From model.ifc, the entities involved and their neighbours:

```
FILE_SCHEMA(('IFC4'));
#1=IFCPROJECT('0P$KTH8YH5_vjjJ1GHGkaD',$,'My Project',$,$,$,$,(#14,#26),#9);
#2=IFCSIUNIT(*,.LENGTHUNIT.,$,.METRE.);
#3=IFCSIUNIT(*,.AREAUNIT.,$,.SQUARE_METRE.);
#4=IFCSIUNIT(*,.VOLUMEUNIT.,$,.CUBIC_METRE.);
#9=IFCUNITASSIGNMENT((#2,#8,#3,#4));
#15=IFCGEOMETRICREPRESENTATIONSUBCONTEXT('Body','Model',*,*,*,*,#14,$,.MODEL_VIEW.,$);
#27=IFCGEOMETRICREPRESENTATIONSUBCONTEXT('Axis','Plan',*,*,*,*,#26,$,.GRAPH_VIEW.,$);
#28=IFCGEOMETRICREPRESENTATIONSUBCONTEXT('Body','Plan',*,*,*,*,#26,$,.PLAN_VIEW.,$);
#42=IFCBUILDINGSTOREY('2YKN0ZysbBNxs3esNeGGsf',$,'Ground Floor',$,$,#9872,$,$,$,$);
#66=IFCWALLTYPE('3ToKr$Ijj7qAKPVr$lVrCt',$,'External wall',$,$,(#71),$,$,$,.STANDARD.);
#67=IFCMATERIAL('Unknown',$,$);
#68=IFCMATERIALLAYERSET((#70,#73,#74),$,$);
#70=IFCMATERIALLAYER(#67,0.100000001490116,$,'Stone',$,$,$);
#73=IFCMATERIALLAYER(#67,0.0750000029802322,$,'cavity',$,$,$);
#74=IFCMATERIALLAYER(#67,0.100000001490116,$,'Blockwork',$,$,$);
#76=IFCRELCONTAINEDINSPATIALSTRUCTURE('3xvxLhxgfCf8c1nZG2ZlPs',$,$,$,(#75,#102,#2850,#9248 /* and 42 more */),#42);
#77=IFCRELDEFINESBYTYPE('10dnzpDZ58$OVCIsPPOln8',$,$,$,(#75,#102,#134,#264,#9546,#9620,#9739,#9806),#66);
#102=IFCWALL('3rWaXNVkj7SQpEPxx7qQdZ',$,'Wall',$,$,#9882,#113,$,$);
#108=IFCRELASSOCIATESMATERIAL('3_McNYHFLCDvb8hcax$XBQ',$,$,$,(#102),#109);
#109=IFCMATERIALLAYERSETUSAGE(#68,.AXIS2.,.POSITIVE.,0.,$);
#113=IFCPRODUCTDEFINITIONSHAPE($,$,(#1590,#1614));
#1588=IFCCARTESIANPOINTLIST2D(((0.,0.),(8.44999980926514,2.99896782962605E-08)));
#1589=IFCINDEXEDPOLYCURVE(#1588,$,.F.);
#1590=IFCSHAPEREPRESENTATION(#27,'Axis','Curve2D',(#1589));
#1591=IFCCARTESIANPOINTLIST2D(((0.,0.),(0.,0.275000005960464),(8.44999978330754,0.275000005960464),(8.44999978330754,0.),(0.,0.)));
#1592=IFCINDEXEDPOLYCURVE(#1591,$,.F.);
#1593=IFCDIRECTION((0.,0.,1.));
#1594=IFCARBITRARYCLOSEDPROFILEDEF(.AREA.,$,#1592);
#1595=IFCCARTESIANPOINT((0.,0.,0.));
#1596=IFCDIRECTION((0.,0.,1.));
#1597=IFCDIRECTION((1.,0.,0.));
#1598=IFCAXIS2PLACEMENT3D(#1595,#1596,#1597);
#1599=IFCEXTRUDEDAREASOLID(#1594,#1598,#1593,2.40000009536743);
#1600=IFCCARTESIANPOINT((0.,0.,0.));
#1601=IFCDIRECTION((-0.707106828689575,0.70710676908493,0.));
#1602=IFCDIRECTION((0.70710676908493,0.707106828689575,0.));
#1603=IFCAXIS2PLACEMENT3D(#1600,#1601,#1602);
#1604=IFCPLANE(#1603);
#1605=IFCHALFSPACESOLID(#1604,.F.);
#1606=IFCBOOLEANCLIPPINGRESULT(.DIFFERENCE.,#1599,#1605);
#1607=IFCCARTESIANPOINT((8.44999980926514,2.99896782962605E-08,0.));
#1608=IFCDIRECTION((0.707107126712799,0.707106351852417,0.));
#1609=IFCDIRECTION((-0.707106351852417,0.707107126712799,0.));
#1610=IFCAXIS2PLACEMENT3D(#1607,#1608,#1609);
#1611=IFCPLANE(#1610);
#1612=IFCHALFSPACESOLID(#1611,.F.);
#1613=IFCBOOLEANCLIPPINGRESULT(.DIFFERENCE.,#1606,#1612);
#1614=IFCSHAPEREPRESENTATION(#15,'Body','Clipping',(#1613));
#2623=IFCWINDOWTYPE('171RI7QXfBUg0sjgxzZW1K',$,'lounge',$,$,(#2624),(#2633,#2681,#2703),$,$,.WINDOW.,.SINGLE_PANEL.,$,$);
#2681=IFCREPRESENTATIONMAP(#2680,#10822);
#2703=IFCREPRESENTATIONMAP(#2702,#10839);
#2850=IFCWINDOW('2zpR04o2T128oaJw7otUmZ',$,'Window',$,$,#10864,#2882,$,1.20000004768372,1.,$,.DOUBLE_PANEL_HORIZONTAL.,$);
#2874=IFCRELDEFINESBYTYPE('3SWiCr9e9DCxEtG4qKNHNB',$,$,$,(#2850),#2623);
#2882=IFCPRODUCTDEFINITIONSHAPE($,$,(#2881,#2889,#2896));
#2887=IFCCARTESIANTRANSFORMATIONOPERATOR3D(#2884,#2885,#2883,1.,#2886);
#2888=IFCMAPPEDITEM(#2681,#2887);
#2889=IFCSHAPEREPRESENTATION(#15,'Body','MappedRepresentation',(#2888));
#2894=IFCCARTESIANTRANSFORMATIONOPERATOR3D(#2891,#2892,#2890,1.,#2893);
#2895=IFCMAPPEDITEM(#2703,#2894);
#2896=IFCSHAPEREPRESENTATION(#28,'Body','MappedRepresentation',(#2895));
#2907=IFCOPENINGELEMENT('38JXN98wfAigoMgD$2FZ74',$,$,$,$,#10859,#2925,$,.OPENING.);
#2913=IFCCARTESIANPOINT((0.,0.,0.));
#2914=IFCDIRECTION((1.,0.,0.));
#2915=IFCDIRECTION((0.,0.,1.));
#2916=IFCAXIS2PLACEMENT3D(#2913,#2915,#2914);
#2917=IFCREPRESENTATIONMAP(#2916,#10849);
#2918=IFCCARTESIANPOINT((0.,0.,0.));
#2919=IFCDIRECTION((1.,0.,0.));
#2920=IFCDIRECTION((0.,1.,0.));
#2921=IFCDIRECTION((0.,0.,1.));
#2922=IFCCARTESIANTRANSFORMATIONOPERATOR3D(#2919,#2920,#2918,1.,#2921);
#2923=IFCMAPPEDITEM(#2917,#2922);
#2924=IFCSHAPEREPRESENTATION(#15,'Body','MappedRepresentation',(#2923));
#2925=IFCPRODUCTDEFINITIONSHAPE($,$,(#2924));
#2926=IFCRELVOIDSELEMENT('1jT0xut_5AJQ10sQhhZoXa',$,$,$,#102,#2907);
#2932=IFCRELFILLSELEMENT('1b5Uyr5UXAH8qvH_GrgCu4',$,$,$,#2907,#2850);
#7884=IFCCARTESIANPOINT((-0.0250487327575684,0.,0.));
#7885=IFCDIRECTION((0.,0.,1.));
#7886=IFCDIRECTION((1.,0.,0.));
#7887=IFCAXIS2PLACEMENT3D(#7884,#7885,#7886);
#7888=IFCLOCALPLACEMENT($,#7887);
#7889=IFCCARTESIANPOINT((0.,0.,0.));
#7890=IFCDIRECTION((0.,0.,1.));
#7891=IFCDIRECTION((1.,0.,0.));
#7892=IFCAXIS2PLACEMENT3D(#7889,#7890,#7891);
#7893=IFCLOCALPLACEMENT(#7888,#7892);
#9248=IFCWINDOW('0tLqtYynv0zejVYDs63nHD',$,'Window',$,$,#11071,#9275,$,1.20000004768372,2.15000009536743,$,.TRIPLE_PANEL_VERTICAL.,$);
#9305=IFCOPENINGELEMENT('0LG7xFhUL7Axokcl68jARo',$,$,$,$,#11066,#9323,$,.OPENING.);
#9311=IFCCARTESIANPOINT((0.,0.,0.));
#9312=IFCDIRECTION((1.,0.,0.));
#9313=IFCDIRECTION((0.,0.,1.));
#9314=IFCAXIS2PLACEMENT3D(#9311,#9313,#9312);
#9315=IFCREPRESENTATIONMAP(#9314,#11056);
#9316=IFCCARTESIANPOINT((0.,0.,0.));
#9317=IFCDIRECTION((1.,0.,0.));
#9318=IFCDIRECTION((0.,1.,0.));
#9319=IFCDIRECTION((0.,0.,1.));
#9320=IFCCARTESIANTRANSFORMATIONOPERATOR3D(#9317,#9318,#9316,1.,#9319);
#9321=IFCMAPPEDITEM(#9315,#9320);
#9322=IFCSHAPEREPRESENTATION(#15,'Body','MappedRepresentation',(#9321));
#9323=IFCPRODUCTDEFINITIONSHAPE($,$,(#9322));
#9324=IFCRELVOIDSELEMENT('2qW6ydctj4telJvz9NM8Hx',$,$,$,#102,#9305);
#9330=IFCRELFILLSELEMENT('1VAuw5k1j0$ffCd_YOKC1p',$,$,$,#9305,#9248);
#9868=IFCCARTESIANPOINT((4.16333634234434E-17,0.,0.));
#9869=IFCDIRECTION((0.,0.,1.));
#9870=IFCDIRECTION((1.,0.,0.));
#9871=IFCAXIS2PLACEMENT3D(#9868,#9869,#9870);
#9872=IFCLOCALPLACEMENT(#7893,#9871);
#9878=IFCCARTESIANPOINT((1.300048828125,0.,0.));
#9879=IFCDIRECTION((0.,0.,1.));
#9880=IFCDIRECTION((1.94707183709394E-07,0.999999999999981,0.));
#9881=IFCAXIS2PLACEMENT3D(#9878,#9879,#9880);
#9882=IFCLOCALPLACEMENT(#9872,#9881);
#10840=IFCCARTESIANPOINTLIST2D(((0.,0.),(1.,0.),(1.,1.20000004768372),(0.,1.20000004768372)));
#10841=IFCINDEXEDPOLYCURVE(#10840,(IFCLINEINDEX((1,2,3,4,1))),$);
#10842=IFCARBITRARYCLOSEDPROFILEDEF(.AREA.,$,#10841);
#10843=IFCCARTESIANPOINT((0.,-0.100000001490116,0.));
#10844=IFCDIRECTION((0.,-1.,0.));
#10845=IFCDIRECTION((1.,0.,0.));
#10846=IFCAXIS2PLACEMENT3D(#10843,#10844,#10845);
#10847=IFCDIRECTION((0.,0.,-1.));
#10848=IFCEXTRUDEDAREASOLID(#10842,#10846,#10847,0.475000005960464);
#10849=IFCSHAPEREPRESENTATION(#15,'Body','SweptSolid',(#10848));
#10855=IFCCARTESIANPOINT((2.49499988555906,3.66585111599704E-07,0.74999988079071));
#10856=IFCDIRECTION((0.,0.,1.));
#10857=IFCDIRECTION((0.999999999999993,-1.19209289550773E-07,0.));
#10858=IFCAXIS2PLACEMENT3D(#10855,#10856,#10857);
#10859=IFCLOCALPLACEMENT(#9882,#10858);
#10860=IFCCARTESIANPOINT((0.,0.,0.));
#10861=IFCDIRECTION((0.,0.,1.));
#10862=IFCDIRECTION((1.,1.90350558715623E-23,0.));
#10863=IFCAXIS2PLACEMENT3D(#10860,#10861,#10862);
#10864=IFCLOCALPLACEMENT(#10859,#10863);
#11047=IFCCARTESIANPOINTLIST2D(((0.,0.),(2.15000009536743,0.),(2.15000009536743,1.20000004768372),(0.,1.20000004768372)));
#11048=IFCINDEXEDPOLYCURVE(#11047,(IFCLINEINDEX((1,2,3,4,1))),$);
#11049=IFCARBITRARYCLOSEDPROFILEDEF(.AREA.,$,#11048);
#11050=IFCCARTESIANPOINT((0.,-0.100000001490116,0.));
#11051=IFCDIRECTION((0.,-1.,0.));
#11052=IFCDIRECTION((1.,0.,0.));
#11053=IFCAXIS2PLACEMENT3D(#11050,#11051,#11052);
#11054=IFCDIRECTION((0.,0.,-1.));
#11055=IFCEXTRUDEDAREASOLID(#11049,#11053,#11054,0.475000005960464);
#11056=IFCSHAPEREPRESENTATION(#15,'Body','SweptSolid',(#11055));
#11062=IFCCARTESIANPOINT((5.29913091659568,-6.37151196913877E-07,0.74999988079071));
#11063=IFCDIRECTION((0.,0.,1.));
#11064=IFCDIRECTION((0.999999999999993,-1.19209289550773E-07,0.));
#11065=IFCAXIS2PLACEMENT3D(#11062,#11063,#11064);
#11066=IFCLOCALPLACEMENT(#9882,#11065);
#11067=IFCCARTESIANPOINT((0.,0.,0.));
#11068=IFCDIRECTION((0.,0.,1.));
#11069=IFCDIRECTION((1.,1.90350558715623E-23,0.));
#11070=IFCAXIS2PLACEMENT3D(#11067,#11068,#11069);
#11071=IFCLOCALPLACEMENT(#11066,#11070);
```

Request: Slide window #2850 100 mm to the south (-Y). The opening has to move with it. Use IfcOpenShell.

```python
import ifcopenshell
import ifcopenshell.api.geometry
import ifcopenshell.util.placement
import ifcopenshell.util.unit

model = ifcopenshell.open("model.ifc")
unit_scale = ifcopenshell.util.unit.calculate_unit_scale(model)

window = model.by_guid("2zpR04o2T128oaJw7otUmZ")
opening = window.FillsVoids[0].RelatingOpeningElement
wall = opening.VoidsElements[0].RelatingBuildingElement

wall_matrix = ifcopenshell.util.placement.get_local_placement(wall.ObjectPlacement)
shift = wall_matrix[:3, 0] * -0.1 / unit_scale
before = ifcopenshell.util.placement.get_local_placement(window.ObjectPlacement)[:3, 3].copy()

# The window is placed relative to its opening, so it follows when the opening moves.
matrix = ifcopenshell.util.placement.get_local_placement(opening.ObjectPlacement)
matrix[:3, 3] += shift
ifcopenshell.api.geometry.edit_object_placement(
    model, product=opening, matrix=matrix, is_si=False, should_transform_children=True
)

after = ifcopenshell.util.placement.get_local_placement(window.ObjectPlacement)[:3, 3]
print("window moved by", (after - before).round(3) + 0.0)

model.write("model_v2.ifc")
```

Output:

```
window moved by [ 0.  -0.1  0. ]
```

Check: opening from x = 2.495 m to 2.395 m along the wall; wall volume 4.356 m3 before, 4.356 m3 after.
